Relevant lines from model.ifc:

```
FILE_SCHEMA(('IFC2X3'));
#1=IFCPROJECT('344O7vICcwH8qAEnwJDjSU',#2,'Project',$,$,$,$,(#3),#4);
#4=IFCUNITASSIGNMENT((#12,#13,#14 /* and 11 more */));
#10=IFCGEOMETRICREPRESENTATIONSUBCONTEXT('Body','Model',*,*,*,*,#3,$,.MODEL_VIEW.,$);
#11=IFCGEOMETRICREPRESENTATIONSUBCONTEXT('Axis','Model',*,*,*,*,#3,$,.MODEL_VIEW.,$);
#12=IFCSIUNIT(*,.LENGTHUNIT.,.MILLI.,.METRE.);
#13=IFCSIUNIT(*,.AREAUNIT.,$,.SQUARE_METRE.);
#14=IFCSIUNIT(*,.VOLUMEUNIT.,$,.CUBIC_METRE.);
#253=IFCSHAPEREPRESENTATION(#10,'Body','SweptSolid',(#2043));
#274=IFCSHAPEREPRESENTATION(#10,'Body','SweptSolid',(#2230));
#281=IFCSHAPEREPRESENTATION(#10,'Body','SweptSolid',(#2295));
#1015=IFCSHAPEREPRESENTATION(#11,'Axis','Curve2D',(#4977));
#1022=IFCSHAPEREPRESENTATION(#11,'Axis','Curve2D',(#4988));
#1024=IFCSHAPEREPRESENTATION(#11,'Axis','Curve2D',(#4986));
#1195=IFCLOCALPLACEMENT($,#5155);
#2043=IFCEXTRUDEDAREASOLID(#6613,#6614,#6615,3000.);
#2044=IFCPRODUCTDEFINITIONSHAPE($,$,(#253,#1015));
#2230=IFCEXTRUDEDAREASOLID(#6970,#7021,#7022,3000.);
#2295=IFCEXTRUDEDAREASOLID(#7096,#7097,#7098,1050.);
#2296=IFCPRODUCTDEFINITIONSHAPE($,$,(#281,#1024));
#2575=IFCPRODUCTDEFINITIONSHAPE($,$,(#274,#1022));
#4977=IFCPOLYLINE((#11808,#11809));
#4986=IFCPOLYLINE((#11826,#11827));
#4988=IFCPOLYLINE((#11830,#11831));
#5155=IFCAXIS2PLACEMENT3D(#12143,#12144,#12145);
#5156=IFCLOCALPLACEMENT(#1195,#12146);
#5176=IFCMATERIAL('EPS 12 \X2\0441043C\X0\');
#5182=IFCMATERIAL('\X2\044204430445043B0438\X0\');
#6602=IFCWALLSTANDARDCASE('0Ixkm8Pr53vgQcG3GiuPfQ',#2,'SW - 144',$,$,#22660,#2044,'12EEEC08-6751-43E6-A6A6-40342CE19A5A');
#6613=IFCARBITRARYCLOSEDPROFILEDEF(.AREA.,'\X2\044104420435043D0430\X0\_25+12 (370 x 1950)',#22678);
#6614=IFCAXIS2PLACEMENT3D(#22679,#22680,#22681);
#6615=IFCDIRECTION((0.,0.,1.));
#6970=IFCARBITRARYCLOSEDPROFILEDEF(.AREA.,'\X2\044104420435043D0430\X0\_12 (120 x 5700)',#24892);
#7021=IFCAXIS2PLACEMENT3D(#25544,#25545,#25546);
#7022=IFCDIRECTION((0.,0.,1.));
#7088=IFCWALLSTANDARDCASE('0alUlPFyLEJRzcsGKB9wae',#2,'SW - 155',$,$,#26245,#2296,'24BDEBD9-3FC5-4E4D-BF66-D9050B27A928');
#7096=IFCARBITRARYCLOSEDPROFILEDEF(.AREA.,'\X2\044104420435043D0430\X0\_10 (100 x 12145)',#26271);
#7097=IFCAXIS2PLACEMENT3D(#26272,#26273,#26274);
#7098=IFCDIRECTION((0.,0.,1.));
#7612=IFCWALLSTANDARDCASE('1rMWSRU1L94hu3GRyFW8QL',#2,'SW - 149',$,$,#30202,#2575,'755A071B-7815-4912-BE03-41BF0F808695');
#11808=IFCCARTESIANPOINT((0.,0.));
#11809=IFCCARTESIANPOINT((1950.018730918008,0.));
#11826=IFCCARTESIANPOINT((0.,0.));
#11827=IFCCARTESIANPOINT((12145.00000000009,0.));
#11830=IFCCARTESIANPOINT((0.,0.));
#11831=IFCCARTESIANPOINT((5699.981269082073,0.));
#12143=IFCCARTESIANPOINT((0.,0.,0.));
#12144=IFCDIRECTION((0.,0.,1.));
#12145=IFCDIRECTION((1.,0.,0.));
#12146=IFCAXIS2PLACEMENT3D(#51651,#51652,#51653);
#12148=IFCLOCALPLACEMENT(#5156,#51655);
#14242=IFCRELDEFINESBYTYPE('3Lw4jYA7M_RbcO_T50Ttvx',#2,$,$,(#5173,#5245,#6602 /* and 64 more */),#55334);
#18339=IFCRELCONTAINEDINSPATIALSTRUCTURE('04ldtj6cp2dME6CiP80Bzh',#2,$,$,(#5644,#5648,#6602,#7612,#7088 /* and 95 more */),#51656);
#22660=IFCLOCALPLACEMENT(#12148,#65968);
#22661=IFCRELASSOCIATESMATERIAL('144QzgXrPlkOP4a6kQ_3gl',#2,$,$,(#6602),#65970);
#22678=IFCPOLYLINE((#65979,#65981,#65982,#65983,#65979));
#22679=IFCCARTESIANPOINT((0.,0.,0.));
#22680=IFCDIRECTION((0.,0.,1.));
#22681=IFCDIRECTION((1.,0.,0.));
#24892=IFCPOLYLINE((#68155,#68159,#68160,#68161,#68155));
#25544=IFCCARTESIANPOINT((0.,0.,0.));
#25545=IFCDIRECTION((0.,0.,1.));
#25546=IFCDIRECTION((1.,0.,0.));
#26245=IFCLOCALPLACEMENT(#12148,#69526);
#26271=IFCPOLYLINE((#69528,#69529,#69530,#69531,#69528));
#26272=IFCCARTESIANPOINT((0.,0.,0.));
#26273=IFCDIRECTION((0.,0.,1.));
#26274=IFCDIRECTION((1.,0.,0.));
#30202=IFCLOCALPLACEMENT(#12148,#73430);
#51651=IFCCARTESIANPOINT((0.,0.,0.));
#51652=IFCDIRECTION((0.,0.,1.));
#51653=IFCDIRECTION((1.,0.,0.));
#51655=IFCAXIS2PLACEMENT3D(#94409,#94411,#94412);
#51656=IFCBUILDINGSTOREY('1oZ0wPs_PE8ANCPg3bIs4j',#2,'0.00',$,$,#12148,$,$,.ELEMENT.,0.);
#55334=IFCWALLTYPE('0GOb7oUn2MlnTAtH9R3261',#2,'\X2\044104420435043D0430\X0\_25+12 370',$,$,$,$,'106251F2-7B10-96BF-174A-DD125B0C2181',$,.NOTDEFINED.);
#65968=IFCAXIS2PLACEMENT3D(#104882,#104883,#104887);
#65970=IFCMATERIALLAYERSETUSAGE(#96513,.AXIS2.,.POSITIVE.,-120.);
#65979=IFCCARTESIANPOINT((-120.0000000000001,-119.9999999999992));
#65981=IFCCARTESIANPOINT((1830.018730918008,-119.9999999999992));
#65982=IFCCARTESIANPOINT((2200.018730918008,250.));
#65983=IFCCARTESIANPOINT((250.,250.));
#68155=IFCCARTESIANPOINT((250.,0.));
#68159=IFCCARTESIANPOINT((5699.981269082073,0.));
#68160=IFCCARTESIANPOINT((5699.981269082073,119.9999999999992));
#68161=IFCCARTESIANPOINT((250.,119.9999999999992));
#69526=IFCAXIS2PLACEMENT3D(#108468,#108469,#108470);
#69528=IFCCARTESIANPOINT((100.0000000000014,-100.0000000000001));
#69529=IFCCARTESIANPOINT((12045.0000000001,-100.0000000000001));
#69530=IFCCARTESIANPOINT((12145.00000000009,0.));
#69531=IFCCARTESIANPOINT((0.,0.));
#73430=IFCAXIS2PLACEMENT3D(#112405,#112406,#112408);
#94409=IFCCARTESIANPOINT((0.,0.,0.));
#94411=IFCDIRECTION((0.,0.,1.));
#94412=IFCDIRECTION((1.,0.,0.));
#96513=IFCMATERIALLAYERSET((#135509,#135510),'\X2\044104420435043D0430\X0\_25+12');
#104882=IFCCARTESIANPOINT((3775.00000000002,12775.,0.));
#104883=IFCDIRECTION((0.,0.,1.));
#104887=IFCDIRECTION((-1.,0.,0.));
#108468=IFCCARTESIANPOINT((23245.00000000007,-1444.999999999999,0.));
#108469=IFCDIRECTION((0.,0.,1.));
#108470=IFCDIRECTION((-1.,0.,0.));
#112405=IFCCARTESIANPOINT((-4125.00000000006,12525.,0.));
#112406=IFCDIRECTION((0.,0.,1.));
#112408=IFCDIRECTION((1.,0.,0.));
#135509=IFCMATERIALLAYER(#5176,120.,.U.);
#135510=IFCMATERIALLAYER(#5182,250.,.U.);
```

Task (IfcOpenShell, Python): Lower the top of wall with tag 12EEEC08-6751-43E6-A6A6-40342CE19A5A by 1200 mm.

```python
import ifcopenshell
import ifcopenshell.geom
import ifcopenshell.util.representation
import ifcopenshell.util.shape

model = ifcopenshell.open("model.ifc")
settings = ifcopenshell.geom.settings()


def volume(element):
    """Net volume in cubic metres, openings subtracted."""
    shape = ifcopenshell.geom.create_shape(settings, element)
    return ifcopenshell.util.shape.get_volume(shape.geometry)


wall = model.by_id(6602)
before = volume(wall)

body = ifcopenshell.util.representation.get_representation(wall, "Model", "Body")
solid = body.Items[0]
old_height = solid.Depth
solid.Depth -= 1200.0
after = volume(wall)

print(f"height {old_height:g} -> {solid.Depth:g}, volume {before:.3f} -> {after:.3f} m3")

model.write("model_edited.ifc")
```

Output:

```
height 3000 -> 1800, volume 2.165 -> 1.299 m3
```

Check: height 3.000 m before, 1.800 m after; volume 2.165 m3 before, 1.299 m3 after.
